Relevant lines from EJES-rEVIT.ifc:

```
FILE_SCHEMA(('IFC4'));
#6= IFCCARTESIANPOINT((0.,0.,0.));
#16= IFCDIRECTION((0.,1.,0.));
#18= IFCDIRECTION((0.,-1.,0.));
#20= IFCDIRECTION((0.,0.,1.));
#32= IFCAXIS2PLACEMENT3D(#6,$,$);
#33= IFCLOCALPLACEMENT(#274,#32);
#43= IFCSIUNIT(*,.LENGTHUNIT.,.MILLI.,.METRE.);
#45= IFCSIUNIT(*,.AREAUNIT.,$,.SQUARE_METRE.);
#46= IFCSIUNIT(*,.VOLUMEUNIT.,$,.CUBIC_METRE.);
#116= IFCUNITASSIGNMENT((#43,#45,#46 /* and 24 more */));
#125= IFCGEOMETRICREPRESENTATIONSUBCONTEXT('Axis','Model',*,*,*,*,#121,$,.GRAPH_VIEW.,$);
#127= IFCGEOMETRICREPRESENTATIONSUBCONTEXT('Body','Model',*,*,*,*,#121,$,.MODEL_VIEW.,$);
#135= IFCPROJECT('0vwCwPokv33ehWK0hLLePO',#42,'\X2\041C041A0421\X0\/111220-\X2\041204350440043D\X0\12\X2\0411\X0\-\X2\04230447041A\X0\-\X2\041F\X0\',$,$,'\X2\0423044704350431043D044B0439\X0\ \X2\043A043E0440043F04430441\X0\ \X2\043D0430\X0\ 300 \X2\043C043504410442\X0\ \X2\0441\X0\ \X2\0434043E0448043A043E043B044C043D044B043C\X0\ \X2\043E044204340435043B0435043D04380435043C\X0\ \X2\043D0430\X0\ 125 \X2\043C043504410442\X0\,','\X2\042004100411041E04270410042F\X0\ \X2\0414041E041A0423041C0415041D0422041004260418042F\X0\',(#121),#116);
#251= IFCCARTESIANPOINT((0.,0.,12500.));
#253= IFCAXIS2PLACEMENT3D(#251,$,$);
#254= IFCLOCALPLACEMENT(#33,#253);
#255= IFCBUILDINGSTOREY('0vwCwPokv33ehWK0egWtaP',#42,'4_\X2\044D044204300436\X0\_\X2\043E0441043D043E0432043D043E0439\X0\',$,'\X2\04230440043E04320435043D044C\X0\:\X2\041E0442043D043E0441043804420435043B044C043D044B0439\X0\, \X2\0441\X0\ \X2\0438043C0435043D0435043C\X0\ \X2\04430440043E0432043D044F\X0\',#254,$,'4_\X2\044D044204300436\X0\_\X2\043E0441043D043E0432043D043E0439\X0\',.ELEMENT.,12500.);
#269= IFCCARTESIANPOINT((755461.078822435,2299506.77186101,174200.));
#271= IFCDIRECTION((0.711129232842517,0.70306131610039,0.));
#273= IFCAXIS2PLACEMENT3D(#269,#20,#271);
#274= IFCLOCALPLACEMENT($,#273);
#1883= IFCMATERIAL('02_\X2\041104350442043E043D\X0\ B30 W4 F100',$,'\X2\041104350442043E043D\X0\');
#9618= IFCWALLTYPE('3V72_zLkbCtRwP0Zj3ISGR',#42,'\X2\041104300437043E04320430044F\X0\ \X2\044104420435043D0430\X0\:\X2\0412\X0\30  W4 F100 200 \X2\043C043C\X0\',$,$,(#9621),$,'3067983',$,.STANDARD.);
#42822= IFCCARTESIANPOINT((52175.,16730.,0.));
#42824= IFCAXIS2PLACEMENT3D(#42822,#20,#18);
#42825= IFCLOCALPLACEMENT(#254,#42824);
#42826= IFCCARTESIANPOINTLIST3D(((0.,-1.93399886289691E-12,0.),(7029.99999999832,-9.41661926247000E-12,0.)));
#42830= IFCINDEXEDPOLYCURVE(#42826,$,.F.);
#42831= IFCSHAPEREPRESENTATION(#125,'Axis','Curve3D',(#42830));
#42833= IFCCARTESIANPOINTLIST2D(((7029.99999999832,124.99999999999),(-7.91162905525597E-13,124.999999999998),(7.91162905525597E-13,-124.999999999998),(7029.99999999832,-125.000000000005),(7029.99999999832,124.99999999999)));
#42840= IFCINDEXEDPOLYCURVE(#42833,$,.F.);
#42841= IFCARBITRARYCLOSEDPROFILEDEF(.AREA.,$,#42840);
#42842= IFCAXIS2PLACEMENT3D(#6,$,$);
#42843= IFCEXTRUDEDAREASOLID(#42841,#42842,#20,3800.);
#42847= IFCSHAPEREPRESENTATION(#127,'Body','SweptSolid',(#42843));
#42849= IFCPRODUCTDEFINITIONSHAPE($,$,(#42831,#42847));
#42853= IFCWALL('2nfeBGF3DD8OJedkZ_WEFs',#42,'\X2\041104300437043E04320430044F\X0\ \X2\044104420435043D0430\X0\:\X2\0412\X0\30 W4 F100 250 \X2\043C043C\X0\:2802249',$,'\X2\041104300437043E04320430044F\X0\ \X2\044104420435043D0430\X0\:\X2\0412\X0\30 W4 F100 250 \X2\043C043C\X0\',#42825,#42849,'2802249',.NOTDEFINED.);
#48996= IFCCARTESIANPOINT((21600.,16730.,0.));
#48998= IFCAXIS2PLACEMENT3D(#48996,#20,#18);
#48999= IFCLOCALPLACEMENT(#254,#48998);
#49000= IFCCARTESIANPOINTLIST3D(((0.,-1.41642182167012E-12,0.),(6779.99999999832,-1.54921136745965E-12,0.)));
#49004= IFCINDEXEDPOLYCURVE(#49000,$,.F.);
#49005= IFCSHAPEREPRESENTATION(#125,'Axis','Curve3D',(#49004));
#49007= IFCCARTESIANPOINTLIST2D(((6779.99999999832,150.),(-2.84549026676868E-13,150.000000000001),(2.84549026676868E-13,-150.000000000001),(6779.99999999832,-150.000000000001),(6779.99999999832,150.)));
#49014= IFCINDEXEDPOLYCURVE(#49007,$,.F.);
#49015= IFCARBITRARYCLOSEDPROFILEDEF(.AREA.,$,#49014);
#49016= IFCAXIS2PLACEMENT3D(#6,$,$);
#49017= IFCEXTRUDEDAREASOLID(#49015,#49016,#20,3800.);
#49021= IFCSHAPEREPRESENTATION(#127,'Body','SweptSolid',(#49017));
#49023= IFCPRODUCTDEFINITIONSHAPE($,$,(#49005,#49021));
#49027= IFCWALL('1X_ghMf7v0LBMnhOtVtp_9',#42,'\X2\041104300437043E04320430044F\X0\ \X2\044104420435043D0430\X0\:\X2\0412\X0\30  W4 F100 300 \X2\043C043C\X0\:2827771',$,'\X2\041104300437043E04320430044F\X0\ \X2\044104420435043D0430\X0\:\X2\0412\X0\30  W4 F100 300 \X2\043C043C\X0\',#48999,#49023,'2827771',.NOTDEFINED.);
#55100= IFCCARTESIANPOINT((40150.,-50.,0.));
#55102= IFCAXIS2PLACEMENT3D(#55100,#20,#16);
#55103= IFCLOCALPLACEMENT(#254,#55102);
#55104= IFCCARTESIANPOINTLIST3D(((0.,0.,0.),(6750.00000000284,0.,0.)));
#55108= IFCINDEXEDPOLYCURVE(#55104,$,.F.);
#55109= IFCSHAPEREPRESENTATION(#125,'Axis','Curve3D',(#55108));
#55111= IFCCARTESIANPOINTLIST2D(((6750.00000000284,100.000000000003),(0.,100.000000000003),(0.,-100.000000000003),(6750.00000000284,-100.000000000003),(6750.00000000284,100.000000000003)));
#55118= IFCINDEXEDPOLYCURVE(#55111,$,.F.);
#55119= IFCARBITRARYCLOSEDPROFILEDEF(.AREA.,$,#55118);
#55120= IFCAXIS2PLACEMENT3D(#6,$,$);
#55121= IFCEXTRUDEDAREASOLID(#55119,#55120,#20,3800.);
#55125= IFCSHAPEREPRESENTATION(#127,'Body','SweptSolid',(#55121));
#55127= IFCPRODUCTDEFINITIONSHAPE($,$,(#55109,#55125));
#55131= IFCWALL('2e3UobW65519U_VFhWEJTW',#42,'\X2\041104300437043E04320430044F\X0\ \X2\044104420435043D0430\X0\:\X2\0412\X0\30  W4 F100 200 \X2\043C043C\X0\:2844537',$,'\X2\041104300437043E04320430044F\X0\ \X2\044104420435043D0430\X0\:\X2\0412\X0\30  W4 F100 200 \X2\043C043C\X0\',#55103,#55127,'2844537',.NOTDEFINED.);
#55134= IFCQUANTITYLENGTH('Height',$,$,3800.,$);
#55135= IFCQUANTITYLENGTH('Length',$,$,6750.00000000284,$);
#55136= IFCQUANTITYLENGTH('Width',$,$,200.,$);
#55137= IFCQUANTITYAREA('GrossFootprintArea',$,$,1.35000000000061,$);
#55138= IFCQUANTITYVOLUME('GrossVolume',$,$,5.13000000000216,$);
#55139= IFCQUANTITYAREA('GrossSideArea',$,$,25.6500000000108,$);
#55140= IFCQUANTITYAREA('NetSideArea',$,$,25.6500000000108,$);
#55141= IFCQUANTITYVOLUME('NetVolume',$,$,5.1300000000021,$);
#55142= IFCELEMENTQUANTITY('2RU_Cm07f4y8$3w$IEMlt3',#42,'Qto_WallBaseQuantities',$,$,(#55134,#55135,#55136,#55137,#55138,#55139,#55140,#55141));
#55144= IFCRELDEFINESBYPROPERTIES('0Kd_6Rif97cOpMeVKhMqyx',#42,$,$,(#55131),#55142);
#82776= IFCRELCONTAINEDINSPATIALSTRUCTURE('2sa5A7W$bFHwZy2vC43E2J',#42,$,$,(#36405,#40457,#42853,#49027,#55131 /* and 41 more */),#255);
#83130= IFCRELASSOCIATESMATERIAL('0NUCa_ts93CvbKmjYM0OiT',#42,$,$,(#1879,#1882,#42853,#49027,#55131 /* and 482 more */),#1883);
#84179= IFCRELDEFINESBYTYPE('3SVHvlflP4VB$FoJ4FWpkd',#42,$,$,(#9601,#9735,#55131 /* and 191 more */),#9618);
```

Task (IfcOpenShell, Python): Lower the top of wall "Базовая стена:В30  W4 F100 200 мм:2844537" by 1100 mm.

```python
import ifcopenshell
import ifcopenshell.api.pset
import ifcopenshell.geom
import ifcopenshell.util.element
import ifcopenshell.util.representation
import ifcopenshell.util.shape
import ifcopenshell.util.unit

model = ifcopenshell.open("EJES-rEVIT.ifc")
unit_scale = ifcopenshell.util.unit.calculate_unit_scale(model)
area_scale = ifcopenshell.util.unit.calculate_unit_scale(model, "AREAUNIT")
volume_scale = ifcopenshell.util.unit.calculate_unit_scale(model, "VOLUMEUNIT")
settings = ifcopenshell.geom.settings()


def volume(element):
    """Net volume in cubic metres, openings subtracted."""
    shape = ifcopenshell.geom.create_shape(settings, element)
    return ifcopenshell.util.shape.get_volume(shape.geometry)


wall = model.by_guid("2e3UobW65519U_VFhWEJTW")
before = volume(wall)

body = ifcopenshell.util.representation.get_representation(wall, "Model", "Body")
solid = body.Items[0]
old_height = solid.Depth
solid.Depth -= 1.1 / unit_scale
after = volume(wall)
thickness = 0.2  # wall thickness in metres

# Update the stored height, areas and volumes.
qto = model.by_id(ifcopenshell.util.element.get_pset(wall, "Qto_WallBaseQuantities", should_inherit=False)["id"])
ifcopenshell.api.pset.edit_qto(model, qto=qto, properties={
    "Height": solid.Depth,
    "GrossVolume": ifcopenshell.util.element.get_pset(wall, "Qto_WallBaseQuantities", "GrossVolume") * solid.Depth / old_height,
    "GrossSideArea": ifcopenshell.util.element.get_pset(wall, "Qto_WallBaseQuantities", "GrossSideArea") * solid.Depth / old_height,
    "NetSideArea": after / thickness / area_scale,
    "NetVolume": after / volume_scale,
})

print(f"height {old_height:g} -> {solid.Depth:g}, volume {before:.3f} -> {after:.3f} m3")

model.write("EJES-rEVIT_edited.ifc")
```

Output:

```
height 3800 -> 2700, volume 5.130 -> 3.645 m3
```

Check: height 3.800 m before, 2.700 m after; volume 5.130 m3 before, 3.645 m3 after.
